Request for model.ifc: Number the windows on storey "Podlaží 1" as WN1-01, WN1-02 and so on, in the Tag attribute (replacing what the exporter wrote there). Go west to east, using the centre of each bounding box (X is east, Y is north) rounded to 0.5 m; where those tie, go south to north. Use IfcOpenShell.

First a look at what the model holds.

```python
import ifcopenshell
import ifcopenshell.util.element
import ifcopenshell.util.placement

model = ifcopenshell.open("model.ifc")
print(model.schema)
storey = next(s for s in model.by_type("IfcBuildingStorey") if s.Name == "Podlaží 1")
windows = [e for e in ifcopenshell.util.element.get_decomposition(storey) if e.is_a("IfcWindow")]
for e in sorted(windows, key=lambda e: e.id()):
    origin = ifcopenshell.util.placement.get_local_placement(e.ObjectPlacement)[:3, 3]
    print(e.id(), e.Tag, e.Name, origin.round(2) + 0.0, sep=" | ")
```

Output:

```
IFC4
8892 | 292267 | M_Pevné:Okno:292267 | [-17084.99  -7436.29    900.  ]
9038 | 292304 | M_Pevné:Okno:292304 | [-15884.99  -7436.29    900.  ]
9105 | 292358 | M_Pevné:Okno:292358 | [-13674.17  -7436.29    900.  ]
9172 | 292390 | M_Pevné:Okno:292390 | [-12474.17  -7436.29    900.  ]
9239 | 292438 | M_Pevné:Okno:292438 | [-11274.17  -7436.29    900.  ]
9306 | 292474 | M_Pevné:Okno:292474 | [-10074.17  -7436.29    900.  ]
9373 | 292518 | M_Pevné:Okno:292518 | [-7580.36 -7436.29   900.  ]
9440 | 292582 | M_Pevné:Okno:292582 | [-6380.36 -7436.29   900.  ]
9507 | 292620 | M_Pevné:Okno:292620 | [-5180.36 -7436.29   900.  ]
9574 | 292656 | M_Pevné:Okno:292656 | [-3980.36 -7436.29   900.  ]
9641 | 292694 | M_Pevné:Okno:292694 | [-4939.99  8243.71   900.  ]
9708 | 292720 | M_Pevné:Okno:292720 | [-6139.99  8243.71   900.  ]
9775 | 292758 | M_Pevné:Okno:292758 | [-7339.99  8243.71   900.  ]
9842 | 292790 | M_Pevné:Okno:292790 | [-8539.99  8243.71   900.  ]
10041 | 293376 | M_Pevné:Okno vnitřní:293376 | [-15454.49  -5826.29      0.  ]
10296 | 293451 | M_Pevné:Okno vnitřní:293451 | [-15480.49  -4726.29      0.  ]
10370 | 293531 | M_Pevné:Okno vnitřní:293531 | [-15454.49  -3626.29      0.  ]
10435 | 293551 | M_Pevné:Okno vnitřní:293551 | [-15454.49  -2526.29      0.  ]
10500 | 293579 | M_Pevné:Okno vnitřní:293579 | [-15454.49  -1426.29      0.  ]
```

```python
import ifcopenshell
import ifcopenshell.geom
import ifcopenshell.util.element
import ifcopenshell.util.shape

model = ifcopenshell.open("model.ifc")
settings = ifcopenshell.geom.settings()
settings.set("use-world-coords", True)


def centre(element):
    shape = ifcopenshell.geom.create_shape(settings, element)
    return ifcopenshell.util.shape.get_bbox_centroid(shape.geometry)


storey = next(s for s in model.by_type("IfcBuildingStorey") if s.Name == "Podlaží 1")
windows = [e for e in ifcopenshell.util.element.get_decomposition(storey) if e.is_a("IfcWindow")]

# Insertion points can sit at a corner or the storey origin, so sort by the geometry (in metres).
centres = {e: centre(e) for e in windows}
windows.sort(key=lambda e: (round(centres[e][0] / 0.5), centres[e][1]))

for i, e in enumerate(windows, start=1):
    number = f"WN1-{i:02d}"
    e.Tag = number
    print(e.id(), number)

model.write("model_edited.ifc")
```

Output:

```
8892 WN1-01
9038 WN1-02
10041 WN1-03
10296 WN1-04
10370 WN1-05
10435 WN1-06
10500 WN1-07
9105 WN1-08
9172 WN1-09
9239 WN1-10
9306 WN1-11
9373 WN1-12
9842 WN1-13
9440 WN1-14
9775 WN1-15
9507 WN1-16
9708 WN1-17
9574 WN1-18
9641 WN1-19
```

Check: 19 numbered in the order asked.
